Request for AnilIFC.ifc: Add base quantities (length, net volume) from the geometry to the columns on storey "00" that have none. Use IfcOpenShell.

First a look at what the model holds.

```python
import ifcopenshell
import ifcopenshell.util.element
import ifcopenshell.util.unit

model = ifcopenshell.open("AnilIFC.ifc")
print(model.schema)
for unit_type in ("LENGTHUNIT", "AREAUNIT", "VOLUMEUNIT"):
    print(unit_type, ifcopenshell.util.unit.calculate_unit_scale(model, unit_type))
storey = next(s for s in model.by_type("IfcBuildingStorey") if s.Name == "00")
columns = [e for e in ifcopenshell.util.element.get_decomposition(storey) if e.is_a("IfcColumn")]
for e in sorted(columns, key=lambda e: e.id()):
    print(e.id(), e.is_a(), e.Name, list(ifcopenshell.util.element.get_psets(e, qtos_only=True)), sep=" | ")
```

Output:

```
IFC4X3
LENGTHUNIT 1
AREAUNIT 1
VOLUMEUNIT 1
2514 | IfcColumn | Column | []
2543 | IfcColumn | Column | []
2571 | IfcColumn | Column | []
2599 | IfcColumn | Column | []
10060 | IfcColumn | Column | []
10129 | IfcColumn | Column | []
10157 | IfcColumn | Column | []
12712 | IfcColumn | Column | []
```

```python
import ifcopenshell
import ifcopenshell.api.pset
import ifcopenshell.geom
import ifcopenshell.util.element
import ifcopenshell.util.shape
import ifcopenshell.util.unit

model = ifcopenshell.open("AnilIFC.ifc")
unit_scale = ifcopenshell.util.unit.calculate_unit_scale(model)
volume_scale = ifcopenshell.util.unit.calculate_unit_scale(model, "VOLUMEUNIT")
settings = ifcopenshell.geom.settings()

storey = next(s for s in model.by_type("IfcBuildingStorey") if s.Name == "00")
columns = [e for e in ifcopenshell.util.element.get_decomposition(storey) if e.is_a("IfcColumn")]

for e in sorted(columns, key=lambda e: e.id()):
    if ifcopenshell.util.element.get_psets(e, qtos_only=True, should_inherit=False):
        continue
    # Geometry comes back in metres, in the element's own axes.
    shape = ifcopenshell.geom.create_shape(settings, e)
    values = {
        "Length": ifcopenshell.util.shape.get_z(shape.geometry) / unit_scale,
        "NetVolume": ifcopenshell.util.shape.get_volume(shape.geometry) / volume_scale,
    }
    qto = ifcopenshell.api.pset.add_qto(model, product=e, name="Qto_ColumnBaseQuantities")
    ifcopenshell.api.pset.edit_qto(model, qto=qto, properties=values)
    print(e.id(), {k: round(v, 3) for k, v in values.items()})

model.write("AnilIFC_v2.ifc")
```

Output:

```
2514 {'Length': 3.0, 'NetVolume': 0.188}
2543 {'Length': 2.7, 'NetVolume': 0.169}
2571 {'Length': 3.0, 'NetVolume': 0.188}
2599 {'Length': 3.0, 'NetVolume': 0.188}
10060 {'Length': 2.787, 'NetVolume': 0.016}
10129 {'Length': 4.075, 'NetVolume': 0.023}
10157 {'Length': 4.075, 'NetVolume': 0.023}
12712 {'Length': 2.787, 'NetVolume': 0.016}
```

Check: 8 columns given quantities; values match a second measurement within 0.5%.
